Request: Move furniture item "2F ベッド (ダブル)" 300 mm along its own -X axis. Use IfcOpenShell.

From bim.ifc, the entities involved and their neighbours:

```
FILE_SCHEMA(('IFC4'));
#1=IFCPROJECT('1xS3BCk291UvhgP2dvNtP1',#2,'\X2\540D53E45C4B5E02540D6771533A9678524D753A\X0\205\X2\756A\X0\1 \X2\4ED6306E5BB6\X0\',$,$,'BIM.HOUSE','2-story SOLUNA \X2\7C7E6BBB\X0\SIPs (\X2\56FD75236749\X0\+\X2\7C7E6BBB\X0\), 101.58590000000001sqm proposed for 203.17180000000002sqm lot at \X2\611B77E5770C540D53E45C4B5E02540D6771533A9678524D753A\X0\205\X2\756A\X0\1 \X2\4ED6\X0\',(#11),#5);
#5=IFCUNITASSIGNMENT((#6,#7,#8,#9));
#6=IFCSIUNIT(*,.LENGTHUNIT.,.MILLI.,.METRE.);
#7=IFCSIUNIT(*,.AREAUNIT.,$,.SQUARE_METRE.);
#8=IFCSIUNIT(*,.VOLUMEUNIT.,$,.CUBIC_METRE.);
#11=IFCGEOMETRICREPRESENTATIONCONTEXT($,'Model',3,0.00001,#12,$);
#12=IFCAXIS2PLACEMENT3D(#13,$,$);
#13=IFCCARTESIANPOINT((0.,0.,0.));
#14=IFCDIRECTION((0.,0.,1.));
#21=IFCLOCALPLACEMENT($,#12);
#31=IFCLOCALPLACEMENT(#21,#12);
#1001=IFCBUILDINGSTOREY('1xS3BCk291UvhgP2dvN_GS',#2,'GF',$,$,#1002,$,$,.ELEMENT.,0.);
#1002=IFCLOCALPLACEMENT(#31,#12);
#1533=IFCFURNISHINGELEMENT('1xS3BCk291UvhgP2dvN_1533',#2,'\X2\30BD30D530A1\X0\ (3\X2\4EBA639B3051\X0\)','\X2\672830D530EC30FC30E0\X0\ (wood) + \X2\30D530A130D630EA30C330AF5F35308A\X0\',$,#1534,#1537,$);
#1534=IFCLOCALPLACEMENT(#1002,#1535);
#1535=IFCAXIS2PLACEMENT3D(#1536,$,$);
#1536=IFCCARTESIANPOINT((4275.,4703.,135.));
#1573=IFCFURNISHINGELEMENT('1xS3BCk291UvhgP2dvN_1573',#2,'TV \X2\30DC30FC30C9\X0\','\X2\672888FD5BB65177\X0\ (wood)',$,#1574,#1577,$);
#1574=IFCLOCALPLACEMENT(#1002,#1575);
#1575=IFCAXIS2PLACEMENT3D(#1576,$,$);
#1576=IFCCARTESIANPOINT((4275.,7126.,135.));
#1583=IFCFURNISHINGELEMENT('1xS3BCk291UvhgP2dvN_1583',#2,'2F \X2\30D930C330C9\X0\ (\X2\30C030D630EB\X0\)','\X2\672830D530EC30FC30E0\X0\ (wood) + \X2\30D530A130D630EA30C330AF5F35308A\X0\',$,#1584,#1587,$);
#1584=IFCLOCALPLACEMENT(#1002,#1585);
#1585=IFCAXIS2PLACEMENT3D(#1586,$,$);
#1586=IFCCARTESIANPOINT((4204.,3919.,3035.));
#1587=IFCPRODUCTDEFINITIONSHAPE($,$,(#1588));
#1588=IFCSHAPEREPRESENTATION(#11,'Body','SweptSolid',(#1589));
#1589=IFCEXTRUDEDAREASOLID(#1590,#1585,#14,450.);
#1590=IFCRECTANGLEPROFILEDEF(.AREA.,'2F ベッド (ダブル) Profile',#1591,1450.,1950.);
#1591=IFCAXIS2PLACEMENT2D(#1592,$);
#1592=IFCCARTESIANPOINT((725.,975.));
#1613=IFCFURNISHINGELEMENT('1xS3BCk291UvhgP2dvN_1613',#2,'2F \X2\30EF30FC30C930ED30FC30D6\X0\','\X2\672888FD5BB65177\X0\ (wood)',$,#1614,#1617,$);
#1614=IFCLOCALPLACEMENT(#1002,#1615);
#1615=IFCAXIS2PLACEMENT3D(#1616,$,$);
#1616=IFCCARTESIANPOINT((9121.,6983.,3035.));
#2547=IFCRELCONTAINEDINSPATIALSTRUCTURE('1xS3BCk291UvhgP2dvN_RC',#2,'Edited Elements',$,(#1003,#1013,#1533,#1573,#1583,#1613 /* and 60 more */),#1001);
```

```python
import ifcopenshell
import ifcopenshell.api.geometry
import ifcopenshell.util.placement
import ifcopenshell.util.unit

model = ifcopenshell.open("bim.ifc")
unit_scale = ifcopenshell.util.unit.calculate_unit_scale(model)

item = model.by_id(1583)
matrix = ifcopenshell.util.placement.get_local_placement(item.ObjectPlacement)
matrix[:3, 3] -= matrix[:3, 0] * 0.3 / unit_scale
ifcopenshell.api.geometry.edit_object_placement(model, product=item, matrix=matrix, is_si=False)

print(ifcopenshell.util.placement.get_local_placement(item.ObjectPlacement).round(3) + 0.0)

model.write("bim_updated.ifc")
```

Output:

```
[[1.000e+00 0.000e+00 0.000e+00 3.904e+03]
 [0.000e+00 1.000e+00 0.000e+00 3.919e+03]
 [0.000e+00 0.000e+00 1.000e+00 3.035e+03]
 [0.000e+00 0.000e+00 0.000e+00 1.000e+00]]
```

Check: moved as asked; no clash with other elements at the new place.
